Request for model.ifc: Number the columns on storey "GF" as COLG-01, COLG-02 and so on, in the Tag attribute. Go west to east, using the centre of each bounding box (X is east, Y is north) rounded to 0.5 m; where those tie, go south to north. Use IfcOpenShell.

First a look at what the model holds.

```python
import ifcopenshell
import ifcopenshell.util.element
import ifcopenshell.util.placement

model = ifcopenshell.open("model.ifc")
print(model.schema)
storey = next(s for s in model.by_type("IfcBuildingStorey") if s.Name == "GF")
columns = [e for e in ifcopenshell.util.element.get_decomposition(storey) if e.is_a("IfcColumn")]
for e in sorted(columns, key=lambda e: e.id()):
    origin = ifcopenshell.util.placement.get_local_placement(e.ObjectPlacement)[:3, 3]
    print(e.id(), e.Tag, e.Name, origin.round(2) + 0.0, sep=" | ")
```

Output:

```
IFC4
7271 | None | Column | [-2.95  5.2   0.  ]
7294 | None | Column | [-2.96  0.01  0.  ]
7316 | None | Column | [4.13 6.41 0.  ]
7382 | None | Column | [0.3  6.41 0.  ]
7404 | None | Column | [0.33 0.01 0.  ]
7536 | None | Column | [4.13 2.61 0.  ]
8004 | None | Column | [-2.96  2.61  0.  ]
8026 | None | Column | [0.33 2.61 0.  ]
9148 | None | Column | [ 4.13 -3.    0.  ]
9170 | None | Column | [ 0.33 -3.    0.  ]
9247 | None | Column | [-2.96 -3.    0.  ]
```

```python
import ifcopenshell
import ifcopenshell.geom
import ifcopenshell.util.element
import ifcopenshell.util.shape

model = ifcopenshell.open("model.ifc")
settings = ifcopenshell.geom.settings()
settings.set("use-world-coords", True)


def centre(element):
    shape = ifcopenshell.geom.create_shape(settings, element)
    return ifcopenshell.util.shape.get_bbox_centroid(shape.geometry)


storey = next(s for s in model.by_type("IfcBuildingStorey") if s.Name == "GF")
columns = [e for e in ifcopenshell.util.element.get_decomposition(storey) if e.is_a("IfcColumn")]

# Insertion points can sit at a corner or the storey origin, so sort by the geometry (in metres).
centres = {e: centre(e) for e in columns}
columns.sort(key=lambda e: (round(centres[e][0] / 0.5), centres[e][1]))

for i, e in enumerate(columns, start=1):
    number = f"COLG-{i:02d}"
    e.Tag = number
    print(e.id(), number)

model.write("model_edited.ifc")
```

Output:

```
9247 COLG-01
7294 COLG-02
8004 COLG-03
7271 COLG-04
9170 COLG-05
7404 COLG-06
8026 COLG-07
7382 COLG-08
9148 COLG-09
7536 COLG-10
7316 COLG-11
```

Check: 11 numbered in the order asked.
